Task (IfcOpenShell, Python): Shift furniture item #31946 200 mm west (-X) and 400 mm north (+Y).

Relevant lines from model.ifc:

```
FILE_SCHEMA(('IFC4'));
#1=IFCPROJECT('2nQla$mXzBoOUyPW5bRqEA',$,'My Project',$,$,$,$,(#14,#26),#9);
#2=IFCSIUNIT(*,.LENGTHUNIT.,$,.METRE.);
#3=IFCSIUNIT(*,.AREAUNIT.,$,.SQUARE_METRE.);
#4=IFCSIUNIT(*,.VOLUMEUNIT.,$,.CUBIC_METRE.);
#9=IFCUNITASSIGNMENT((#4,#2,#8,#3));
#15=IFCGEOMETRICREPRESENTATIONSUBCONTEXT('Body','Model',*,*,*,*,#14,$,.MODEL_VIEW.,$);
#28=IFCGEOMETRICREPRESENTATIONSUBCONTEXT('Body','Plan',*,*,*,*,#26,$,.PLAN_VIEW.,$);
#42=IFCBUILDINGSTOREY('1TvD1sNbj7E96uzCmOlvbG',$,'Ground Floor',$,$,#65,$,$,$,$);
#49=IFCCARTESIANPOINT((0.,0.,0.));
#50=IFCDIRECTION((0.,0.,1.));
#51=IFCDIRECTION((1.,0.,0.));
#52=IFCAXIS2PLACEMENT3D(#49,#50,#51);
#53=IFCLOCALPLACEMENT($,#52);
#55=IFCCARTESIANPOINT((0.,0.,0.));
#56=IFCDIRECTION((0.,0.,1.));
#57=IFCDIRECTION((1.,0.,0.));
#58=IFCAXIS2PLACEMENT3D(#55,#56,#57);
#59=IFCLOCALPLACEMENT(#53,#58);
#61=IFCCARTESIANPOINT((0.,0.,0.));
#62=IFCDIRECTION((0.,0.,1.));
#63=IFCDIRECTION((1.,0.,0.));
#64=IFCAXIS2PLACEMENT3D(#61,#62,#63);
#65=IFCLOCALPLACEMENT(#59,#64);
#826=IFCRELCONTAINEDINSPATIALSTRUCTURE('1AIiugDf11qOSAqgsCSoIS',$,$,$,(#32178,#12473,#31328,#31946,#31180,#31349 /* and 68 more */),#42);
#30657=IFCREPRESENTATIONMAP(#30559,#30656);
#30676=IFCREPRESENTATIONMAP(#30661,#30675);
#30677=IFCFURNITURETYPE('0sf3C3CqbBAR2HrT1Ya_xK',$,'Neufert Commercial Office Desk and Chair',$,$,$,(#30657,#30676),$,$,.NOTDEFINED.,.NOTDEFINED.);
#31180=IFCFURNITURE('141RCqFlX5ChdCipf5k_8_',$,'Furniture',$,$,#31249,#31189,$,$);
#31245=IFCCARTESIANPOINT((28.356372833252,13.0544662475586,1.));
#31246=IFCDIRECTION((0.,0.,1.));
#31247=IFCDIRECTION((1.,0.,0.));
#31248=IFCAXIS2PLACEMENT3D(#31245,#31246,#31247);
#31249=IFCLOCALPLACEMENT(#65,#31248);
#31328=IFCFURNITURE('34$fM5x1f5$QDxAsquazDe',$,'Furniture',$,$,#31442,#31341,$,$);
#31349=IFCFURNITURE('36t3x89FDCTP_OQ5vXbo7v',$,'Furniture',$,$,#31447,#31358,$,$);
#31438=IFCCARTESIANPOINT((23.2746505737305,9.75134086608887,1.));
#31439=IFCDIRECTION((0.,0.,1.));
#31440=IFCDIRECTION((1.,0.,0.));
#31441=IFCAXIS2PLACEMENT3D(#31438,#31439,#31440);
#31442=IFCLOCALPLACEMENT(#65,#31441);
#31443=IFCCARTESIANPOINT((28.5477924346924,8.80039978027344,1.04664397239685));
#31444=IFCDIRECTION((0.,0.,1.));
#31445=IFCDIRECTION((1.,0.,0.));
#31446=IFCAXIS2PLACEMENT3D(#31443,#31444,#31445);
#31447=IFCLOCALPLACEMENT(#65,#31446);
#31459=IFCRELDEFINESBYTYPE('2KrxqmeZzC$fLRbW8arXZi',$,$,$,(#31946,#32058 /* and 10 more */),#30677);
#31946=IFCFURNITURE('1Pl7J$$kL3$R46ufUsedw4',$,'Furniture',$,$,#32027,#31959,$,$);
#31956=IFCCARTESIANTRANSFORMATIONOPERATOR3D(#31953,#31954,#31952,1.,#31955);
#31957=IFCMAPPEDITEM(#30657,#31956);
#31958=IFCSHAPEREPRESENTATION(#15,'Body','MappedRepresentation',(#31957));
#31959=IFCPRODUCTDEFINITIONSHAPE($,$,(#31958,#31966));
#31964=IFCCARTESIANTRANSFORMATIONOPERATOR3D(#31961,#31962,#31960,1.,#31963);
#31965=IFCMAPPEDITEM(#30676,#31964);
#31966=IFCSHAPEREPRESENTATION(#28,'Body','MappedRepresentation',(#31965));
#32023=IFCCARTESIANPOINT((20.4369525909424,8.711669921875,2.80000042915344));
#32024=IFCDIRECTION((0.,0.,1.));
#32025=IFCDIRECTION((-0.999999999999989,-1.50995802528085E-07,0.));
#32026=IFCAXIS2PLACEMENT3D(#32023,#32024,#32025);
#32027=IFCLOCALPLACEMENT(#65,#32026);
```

```python
import ifcopenshell
import ifcopenshell.api.geometry
import ifcopenshell.util.placement

model = ifcopenshell.open("model.ifc")

item = model.by_guid("1Pl7J$$kL3$R46ufUsedw4")
matrix = ifcopenshell.util.placement.get_local_placement(item.ObjectPlacement)
matrix[0, 3] -= 0.2
matrix[1, 3] += 0.4
ifcopenshell.api.geometry.edit_object_placement(model, product=item, matrix=matrix, is_si=False)

print(ifcopenshell.util.placement.get_local_placement(item.ObjectPlacement).round(3) + 0.0)

model.write("model_edited.ifc")
```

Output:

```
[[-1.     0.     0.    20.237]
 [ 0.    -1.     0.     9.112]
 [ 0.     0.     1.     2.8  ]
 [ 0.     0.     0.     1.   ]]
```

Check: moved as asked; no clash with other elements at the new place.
